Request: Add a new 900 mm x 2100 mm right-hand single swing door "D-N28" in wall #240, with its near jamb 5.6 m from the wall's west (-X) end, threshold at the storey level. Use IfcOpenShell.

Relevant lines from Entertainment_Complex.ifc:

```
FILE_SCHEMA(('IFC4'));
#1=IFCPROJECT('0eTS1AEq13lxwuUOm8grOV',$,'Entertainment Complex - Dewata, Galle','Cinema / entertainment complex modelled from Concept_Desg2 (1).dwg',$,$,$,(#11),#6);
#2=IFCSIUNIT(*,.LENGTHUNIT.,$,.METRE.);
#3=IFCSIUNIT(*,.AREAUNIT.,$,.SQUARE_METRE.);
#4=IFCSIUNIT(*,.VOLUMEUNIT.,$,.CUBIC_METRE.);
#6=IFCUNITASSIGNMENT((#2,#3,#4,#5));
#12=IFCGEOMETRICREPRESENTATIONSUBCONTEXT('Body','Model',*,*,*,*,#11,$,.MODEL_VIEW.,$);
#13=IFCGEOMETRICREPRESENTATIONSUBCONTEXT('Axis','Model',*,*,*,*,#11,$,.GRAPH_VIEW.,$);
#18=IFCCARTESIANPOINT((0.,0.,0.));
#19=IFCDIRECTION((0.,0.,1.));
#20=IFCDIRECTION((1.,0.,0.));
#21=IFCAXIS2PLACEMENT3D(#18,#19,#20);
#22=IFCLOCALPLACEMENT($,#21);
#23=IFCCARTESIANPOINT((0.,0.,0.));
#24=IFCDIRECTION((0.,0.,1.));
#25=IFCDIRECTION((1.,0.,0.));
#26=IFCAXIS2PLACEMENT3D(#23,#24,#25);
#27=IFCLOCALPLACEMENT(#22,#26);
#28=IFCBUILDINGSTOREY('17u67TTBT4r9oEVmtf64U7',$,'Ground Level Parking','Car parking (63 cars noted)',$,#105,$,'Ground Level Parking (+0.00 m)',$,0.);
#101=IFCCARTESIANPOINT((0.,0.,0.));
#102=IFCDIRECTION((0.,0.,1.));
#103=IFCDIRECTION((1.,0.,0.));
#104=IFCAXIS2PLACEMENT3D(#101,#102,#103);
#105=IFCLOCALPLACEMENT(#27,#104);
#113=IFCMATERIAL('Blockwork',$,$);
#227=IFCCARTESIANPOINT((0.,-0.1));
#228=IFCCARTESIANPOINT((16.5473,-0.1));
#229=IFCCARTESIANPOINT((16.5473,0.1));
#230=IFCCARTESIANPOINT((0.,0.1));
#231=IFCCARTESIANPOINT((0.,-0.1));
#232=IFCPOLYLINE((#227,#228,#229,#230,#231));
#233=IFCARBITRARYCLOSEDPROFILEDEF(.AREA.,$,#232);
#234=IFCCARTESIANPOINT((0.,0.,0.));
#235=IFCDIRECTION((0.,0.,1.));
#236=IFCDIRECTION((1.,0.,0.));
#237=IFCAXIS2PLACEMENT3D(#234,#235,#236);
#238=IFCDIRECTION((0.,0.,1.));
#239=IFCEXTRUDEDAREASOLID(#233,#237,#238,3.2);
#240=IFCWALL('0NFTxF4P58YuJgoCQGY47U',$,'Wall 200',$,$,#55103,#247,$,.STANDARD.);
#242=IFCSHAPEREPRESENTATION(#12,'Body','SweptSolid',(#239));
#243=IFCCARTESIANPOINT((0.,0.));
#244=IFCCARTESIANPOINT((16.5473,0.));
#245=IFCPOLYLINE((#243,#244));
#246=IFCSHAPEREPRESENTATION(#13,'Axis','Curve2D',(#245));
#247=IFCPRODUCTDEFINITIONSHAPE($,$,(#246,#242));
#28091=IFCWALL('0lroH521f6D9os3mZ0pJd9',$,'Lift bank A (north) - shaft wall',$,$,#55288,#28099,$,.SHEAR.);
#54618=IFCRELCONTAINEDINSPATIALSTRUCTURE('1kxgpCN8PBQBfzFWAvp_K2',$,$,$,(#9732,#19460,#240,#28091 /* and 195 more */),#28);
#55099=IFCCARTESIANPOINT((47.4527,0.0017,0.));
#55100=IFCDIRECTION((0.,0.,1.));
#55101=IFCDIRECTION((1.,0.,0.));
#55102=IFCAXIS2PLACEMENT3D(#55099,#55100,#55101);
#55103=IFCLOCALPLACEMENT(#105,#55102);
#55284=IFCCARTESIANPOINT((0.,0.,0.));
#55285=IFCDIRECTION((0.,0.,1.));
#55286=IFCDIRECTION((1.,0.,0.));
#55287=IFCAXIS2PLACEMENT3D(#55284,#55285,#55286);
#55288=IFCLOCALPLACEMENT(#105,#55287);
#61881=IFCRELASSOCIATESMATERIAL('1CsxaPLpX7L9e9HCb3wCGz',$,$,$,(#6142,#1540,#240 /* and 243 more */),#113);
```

```python
import numpy as np
import ifcopenshell
import ifcopenshell.api.feature
import ifcopenshell.api.geometry
import ifcopenshell.api.root
import ifcopenshell.api.spatial
import ifcopenshell.geom
import ifcopenshell.util.element
import ifcopenshell.util.placement
import ifcopenshell.util.representation
import ifcopenshell.util.shape
import ifcopenshell.util.unit

model = ifcopenshell.open("Entertainment_Complex.ifc")
unit_scale = ifcopenshell.util.unit.calculate_unit_scale(model)
settings = ifcopenshell.geom.settings()


def volume(element):
    """Net volume in cubic metres, openings subtracted."""
    shape = ifcopenshell.geom.create_shape(settings, element)
    return ifcopenshell.util.shape.get_volume(shape.geometry)


wall = model.by_id(240)
storey = ifcopenshell.util.element.get_container(wall, ifc_class="IfcBuildingStorey")
context = ifcopenshell.util.representation.get_context(model, "Model", "Body", "MODEL_VIEW")
before = volume(wall)

width, height, from_end, sill = 0.9, 2.1, 5.6, 0.0  # metres

# The wall runs along its own X axis, and the end named is its -X end.
wall_shape = ifcopenshell.geom.create_shape(settings, wall)
x, y, z = ifcopenshell.util.shape.get_vertices(wall_shape.geometry).T
start = x.min() + from_end
face, thickness = float(y.min()), float(y.max() - y.min())
wall_matrix = ifcopenshell.util.placement.get_local_placement(wall.ObjectPlacement)
level = ifcopenshell.util.placement.get_local_placement(storey.ObjectPlacement)[2, 3]


def in_wall(x, y):
    """Placement at x, y metres in the wall's axes, at sill height."""
    matrix = wall_matrix.copy()
    matrix[:, 3] = wall_matrix @ np.array([x / unit_scale, y / unit_scale, 0.0, 1.0])
    matrix[2, 3] = level + sill / unit_scale
    return matrix


# Opening: a box that overshoots both wall faces by 50 mm.
opening = ifcopenshell.api.root.create_entity(model, ifc_class="IfcOpeningElement", predefined_type="OPENING")
box = ifcopenshell.api.geometry.add_wall_representation(
    model, context=context, length=width, height=height, thickness=thickness + 0.1
)
ifcopenshell.api.geometry.assign_representation(model, product=opening, representation=box)
ifcopenshell.api.geometry.edit_object_placement(model, product=opening, matrix=in_wall(start, face - 0.05), is_si=False)
ifcopenshell.api.feature.add_feature(model, feature=opening, element=wall)

door = ifcopenshell.api.root.create_entity(model, ifc_class="IfcDoor", name="D-N28", predefined_type="DOOR")
door.OverallWidth, door.OverallHeight = width / unit_scale, height / unit_scale
door.OperationType = "SINGLE_SWING_RIGHT"
body = ifcopenshell.api.geometry.add_door_representation(
    model,
    context=context,
    overall_width=door.OverallWidth,
    overall_height=door.OverallHeight,
    operation_type="SINGLE_SWING_RIGHT",
    lining_properties={"LiningDepth": thickness / unit_scale, "ThresholdDepth": thickness / unit_scale},
)
ifcopenshell.api.geometry.assign_representation(model, product=door, representation=body)
ifcopenshell.api.spatial.assign_container(model, products=[door], relating_structure=storey)
ifcopenshell.api.feature.add_filling(model, opening=opening, element=door)

# The lining spans the wall, so the door starts at the wall face.
ifcopenshell.api.geometry.edit_object_placement(model, product=door, matrix=in_wall(start, face), is_si=False)

after = volume(wall)

print(f"wall volume {before:.3f} -> {after:.3f} m3")

model.write("Entertainment_Complex_edited.ifc")
```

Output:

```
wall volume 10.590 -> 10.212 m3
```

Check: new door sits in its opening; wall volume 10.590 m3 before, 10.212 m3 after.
